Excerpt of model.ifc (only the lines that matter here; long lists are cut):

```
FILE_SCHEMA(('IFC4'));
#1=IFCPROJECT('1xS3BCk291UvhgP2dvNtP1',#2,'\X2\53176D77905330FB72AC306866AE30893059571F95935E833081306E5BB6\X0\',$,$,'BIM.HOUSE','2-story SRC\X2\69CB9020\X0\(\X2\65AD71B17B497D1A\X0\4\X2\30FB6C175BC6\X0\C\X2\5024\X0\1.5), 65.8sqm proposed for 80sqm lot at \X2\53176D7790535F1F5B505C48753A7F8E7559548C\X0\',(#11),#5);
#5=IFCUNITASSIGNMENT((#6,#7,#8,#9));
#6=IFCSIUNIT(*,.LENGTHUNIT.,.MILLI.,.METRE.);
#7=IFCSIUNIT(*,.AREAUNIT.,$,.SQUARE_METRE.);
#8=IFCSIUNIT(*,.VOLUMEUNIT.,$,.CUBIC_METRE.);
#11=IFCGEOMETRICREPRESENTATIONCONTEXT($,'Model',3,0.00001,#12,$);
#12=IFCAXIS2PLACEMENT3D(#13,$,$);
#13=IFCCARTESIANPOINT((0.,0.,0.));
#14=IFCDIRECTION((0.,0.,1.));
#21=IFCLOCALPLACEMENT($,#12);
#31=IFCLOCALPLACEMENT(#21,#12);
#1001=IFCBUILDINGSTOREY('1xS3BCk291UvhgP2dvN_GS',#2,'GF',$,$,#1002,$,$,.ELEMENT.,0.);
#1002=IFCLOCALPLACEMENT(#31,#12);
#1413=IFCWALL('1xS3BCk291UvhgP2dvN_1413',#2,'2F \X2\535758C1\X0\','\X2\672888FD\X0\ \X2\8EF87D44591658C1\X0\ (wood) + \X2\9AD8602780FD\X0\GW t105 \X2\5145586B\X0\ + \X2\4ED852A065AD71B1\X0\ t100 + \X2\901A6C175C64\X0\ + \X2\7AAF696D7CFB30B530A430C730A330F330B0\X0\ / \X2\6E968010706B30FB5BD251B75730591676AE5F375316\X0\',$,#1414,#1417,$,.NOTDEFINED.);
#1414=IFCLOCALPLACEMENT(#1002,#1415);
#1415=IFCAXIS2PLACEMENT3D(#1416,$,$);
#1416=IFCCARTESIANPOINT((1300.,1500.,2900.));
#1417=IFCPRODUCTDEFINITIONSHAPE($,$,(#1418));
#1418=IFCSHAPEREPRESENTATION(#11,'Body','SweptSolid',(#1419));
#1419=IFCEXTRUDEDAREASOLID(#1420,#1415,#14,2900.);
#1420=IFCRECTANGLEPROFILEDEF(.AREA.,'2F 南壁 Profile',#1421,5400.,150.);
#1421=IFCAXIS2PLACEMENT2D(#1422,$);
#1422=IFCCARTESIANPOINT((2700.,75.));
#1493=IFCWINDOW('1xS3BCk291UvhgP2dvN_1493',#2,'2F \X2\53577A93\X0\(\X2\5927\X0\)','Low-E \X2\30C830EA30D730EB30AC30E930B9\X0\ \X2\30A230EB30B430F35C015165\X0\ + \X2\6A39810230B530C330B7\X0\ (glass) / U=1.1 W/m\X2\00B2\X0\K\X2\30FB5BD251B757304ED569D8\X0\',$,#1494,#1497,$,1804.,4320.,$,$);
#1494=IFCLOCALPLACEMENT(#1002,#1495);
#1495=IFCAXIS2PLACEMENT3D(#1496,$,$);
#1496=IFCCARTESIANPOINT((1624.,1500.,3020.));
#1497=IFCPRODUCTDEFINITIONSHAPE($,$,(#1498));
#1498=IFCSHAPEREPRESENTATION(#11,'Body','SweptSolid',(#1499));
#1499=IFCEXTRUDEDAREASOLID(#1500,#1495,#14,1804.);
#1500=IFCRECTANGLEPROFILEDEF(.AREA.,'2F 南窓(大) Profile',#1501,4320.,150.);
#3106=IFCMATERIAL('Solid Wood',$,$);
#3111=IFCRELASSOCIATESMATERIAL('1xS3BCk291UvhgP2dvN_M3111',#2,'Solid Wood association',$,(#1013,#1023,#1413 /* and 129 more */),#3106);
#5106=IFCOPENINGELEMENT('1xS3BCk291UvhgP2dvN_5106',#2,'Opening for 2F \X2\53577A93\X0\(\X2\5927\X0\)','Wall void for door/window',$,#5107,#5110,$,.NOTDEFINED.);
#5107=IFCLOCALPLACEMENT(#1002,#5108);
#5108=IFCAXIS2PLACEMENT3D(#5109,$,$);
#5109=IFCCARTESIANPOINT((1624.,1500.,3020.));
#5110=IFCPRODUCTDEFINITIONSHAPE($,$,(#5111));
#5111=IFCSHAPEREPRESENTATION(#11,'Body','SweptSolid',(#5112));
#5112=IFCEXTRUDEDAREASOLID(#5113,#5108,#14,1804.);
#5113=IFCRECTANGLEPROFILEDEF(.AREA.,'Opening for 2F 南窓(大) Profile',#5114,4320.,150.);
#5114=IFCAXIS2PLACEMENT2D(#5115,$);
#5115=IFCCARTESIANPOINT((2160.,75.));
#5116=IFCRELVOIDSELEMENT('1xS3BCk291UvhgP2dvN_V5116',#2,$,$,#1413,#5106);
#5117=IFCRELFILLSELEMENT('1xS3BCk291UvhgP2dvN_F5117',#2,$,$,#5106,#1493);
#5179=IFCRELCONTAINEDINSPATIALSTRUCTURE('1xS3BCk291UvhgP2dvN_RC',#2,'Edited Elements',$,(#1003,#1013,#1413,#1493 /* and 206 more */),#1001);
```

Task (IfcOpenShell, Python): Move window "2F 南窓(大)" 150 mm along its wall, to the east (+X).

```python
import ifcopenshell
import ifcopenshell.api.geometry
import ifcopenshell.util.placement
import ifcopenshell.util.unit

model = ifcopenshell.open("model.ifc")
unit_scale = ifcopenshell.util.unit.calculate_unit_scale(model)

window = model.by_id(1493)
opening = window.FillsVoids[0].RelatingOpeningElement
wall = opening.VoidsElements[0].RelatingBuildingElement

wall_matrix = ifcopenshell.util.placement.get_local_placement(wall.ObjectPlacement)
shift = wall_matrix[:3, 0] * 0.15 / unit_scale
before = ifcopenshell.util.placement.get_local_placement(window.ObjectPlacement)[:3, 3].copy()

# The window is not placed relative to its opening, so move both.
for product in (opening, window):
    matrix = ifcopenshell.util.placement.get_local_placement(product.ObjectPlacement)
    matrix[:3, 3] += shift
    ifcopenshell.api.geometry.edit_object_placement(model, product=product, matrix=matrix, is_si=False)

after = ifcopenshell.util.placement.get_local_placement(window.ObjectPlacement)[:3, 3]
print("window moved by", (after - before).round(3) + 0.0)

model.write("model_edited.ifc")
```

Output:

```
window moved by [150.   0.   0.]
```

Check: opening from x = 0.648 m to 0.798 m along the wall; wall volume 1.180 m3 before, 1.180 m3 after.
